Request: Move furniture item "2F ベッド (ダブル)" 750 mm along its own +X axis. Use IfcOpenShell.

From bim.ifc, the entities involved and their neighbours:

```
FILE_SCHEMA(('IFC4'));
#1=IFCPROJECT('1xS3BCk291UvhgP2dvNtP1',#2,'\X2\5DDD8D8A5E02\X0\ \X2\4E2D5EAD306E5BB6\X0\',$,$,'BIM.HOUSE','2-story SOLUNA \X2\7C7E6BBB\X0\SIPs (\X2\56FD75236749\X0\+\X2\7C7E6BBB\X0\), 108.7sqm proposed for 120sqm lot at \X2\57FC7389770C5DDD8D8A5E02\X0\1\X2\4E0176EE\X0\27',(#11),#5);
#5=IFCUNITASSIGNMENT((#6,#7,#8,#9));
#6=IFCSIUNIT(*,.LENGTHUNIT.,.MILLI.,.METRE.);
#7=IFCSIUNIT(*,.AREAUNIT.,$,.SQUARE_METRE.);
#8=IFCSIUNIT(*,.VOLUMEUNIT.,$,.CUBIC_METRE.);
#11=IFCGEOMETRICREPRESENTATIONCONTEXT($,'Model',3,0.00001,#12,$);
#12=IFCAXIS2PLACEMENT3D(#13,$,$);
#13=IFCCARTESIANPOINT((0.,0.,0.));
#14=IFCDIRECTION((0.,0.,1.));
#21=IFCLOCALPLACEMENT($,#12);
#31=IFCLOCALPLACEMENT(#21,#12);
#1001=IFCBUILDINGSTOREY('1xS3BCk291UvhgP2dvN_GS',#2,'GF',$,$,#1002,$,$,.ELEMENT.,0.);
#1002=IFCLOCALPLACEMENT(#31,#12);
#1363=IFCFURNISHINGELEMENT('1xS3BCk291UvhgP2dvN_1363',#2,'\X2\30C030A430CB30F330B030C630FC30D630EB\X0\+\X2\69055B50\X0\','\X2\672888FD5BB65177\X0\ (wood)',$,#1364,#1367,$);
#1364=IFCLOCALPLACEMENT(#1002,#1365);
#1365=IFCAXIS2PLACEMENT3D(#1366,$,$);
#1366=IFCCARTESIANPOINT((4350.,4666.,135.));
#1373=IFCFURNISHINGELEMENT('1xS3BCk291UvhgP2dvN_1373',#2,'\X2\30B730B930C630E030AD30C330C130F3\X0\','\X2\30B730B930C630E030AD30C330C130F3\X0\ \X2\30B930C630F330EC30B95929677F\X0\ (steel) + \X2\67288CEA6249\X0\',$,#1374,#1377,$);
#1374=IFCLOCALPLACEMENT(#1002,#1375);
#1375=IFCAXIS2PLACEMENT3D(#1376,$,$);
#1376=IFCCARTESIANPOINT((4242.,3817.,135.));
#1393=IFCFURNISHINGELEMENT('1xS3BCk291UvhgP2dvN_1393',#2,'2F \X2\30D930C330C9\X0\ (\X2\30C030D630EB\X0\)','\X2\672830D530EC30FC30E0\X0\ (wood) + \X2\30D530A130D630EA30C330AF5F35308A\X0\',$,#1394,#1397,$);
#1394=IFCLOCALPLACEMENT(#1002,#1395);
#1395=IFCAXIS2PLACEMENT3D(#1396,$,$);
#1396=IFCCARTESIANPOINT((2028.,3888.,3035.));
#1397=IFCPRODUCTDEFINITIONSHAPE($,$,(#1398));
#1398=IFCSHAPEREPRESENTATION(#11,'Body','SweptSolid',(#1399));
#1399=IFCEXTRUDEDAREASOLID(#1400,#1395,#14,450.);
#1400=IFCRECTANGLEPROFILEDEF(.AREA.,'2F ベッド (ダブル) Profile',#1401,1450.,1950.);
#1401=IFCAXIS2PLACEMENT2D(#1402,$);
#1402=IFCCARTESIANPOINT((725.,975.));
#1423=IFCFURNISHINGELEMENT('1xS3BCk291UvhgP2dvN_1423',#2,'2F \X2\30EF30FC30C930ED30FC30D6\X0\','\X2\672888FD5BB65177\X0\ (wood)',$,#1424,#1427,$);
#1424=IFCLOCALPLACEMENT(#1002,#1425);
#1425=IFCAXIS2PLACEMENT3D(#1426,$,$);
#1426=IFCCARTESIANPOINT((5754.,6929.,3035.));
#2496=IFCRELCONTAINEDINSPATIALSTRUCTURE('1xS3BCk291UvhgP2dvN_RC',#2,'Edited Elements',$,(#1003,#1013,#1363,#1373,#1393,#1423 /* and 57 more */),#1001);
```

```python
import ifcopenshell
import ifcopenshell.api.geometry
import ifcopenshell.util.placement
import ifcopenshell.util.unit

model = ifcopenshell.open("bim.ifc")
unit_scale = ifcopenshell.util.unit.calculate_unit_scale(model)

item = model.by_guid("1xS3BCk291UvhgP2dvN_1393")
matrix = ifcopenshell.util.placement.get_local_placement(item.ObjectPlacement)
matrix[:3, 3] += matrix[:3, 0] * 0.75 / unit_scale
ifcopenshell.api.geometry.edit_object_placement(model, product=item, matrix=matrix, is_si=False)

print(ifcopenshell.util.placement.get_local_placement(item.ObjectPlacement).round(3) + 0.0)

model.write("bim_updated.ifc")
```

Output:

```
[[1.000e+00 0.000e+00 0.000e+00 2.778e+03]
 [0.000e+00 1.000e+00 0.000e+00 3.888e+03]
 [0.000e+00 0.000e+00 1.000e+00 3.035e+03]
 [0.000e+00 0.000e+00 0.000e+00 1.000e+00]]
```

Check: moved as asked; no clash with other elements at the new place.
